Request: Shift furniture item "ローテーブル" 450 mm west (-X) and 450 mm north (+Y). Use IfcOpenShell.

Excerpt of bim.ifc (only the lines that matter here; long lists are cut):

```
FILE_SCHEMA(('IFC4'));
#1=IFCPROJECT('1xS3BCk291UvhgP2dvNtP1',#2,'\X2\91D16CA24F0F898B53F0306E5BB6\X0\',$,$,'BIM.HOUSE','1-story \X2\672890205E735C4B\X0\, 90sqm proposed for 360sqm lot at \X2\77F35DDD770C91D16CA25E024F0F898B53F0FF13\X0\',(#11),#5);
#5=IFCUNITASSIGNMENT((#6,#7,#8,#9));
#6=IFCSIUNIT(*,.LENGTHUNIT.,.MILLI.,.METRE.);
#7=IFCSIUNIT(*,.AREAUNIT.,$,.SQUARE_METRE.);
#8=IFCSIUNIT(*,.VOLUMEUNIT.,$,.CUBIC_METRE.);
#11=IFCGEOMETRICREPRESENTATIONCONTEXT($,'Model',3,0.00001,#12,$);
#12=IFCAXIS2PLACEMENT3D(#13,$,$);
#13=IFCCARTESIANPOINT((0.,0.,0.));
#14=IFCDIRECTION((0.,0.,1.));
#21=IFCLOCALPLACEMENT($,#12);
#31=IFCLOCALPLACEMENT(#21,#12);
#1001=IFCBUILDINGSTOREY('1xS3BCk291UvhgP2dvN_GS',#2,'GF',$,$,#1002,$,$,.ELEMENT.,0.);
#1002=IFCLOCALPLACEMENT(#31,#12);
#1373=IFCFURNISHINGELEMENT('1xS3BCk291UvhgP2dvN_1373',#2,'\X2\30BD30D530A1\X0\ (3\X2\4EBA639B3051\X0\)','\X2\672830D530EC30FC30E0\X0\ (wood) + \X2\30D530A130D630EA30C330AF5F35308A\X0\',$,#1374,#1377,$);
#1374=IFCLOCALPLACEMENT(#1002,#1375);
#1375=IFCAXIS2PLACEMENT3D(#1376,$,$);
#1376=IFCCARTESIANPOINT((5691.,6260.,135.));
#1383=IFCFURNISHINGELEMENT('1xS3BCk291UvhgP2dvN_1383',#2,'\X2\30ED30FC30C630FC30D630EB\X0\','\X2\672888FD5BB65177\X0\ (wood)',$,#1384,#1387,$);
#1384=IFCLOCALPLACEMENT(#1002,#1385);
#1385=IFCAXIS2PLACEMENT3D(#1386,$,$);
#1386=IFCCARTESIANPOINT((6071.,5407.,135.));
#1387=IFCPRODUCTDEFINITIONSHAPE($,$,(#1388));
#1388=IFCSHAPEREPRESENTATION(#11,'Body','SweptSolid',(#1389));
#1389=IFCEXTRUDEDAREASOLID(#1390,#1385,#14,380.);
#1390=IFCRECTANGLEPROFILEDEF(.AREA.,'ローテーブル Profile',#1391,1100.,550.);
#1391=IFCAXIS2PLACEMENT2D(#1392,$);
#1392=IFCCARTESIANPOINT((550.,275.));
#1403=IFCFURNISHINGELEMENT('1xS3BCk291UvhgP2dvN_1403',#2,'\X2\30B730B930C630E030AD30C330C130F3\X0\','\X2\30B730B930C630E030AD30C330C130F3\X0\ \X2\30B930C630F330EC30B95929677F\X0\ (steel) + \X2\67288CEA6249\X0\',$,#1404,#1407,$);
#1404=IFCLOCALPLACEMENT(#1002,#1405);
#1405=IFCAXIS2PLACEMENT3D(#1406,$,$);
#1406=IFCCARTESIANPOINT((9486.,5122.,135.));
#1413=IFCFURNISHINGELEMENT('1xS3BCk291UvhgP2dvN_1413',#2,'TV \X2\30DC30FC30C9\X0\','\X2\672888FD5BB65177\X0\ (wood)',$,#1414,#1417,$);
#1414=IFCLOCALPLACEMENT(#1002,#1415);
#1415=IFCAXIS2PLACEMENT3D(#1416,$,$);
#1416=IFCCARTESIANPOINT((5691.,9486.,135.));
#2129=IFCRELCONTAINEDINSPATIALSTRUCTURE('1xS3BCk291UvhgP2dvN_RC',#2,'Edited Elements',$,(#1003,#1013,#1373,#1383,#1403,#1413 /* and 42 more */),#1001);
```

```python
import ifcopenshell
import ifcopenshell.api.geometry
import ifcopenshell.util.placement

model = ifcopenshell.open("bim.ifc")

item = model.by_id(1383)
matrix = ifcopenshell.util.placement.get_local_placement(item.ObjectPlacement)
matrix[0, 3] -= 450.0
matrix[1, 3] += 450.0
ifcopenshell.api.geometry.edit_object_placement(model, product=item, matrix=matrix, is_si=False)

print(ifcopenshell.util.placement.get_local_placement(item.ObjectPlacement).round(3) + 0.0)

model.write("bim_updated.ifc")
```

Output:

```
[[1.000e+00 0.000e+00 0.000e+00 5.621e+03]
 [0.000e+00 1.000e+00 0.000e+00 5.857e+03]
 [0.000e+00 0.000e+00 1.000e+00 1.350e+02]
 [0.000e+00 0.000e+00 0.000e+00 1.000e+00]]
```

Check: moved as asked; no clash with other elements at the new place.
